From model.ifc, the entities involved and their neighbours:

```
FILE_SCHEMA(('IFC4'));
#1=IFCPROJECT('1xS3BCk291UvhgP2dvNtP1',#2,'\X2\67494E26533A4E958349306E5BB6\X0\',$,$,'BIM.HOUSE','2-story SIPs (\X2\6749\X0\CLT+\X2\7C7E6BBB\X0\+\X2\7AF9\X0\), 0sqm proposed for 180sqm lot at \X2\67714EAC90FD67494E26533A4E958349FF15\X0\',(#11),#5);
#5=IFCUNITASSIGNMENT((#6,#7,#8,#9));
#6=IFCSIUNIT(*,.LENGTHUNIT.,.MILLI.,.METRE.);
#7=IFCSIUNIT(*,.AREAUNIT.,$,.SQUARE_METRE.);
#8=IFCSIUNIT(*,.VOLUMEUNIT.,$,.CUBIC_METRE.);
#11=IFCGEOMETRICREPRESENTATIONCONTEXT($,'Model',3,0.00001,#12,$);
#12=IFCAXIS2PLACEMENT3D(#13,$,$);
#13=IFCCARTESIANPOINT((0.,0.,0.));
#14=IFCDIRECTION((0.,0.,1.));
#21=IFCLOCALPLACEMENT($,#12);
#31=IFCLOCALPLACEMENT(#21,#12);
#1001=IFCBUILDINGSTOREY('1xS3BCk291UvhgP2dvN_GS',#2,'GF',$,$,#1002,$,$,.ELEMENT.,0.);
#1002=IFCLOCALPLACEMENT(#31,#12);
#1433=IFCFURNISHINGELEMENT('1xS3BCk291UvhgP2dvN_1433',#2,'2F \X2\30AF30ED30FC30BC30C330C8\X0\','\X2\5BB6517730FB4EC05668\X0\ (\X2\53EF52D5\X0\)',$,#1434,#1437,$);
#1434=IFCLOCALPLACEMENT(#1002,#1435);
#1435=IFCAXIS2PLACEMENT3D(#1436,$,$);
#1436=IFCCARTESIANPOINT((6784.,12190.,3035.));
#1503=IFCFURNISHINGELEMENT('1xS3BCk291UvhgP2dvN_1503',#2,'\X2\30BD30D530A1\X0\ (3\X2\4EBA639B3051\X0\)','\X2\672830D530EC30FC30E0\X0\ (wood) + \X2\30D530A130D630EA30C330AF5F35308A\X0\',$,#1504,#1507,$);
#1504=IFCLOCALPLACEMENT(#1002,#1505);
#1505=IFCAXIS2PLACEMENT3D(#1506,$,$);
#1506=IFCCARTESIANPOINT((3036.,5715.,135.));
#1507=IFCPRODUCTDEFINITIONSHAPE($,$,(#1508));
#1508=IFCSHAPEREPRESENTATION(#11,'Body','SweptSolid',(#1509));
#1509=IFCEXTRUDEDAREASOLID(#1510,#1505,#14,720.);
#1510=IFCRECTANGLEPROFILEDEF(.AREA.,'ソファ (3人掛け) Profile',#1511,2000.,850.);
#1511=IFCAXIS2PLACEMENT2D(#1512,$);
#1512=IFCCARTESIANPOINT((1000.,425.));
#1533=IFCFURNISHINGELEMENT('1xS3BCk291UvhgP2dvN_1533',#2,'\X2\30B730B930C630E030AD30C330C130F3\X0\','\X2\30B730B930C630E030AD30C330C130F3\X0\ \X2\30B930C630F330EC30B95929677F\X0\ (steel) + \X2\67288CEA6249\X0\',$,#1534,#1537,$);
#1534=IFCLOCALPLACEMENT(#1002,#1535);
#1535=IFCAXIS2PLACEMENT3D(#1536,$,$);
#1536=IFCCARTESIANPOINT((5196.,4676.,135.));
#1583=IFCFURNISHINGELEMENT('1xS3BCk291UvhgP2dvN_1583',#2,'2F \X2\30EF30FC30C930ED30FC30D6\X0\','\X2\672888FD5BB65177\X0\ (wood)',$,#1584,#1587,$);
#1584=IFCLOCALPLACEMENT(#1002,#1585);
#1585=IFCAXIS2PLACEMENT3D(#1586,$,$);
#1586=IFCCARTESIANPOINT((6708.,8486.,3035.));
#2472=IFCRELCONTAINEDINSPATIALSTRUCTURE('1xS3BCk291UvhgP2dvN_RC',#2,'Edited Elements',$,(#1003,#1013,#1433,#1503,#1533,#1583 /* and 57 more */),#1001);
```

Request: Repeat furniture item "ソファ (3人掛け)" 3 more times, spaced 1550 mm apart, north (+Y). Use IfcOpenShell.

```python
import numpy as np
import ifcopenshell
import ifcopenshell.api.geometry
import ifcopenshell.api.root
import ifcopenshell.util.element
import ifcopenshell.util.placement
import ifcopenshell.util.unit

model = ifcopenshell.open("model.ifc")
unit_scale = ifcopenshell.util.unit.calculate_unit_scale(model)


def reuse_history(source, copy):
    """copy_class also copies each property set's owner history, people and application; keep the originals."""
    for rel in copy.IsDefinedBy:
        if rel.is_a("IfcRelDefinesByProperties") and (history := rel.RelatingPropertyDefinition.OwnerHistory):
            rel.RelatingPropertyDefinition.OwnerHistory = source.OwnerHistory
            ifcopenshell.util.element.remove_deep2(model, history)


source = model.by_id(1503)
base = ifcopenshell.util.placement.get_local_placement(source.ObjectPlacement)
step = np.array([0.0, 1.0, 0.0]) * 1.55 / unit_scale

for i in range(1, 4):
    copy = ifcopenshell.api.root.copy_class(model, product=source)
    copy.Representation = ifcopenshell.util.element.copy_deep(
        model, source.Representation, exclude=["IfcGeometricRepresentationContext", "IfcRepresentationMap"]
    )
    reuse_history(source, copy)
    matrix = base.copy()
    matrix[:3, 3] += i * step
    print("added at", matrix[:3, 3].round(3) + 0.0)
    ifcopenshell.api.geometry.edit_object_placement(model, product=copy, matrix=matrix, is_si=False)

model.write("model_edited.ifc")
```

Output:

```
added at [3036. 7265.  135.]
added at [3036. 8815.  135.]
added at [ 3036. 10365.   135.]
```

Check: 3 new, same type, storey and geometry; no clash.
